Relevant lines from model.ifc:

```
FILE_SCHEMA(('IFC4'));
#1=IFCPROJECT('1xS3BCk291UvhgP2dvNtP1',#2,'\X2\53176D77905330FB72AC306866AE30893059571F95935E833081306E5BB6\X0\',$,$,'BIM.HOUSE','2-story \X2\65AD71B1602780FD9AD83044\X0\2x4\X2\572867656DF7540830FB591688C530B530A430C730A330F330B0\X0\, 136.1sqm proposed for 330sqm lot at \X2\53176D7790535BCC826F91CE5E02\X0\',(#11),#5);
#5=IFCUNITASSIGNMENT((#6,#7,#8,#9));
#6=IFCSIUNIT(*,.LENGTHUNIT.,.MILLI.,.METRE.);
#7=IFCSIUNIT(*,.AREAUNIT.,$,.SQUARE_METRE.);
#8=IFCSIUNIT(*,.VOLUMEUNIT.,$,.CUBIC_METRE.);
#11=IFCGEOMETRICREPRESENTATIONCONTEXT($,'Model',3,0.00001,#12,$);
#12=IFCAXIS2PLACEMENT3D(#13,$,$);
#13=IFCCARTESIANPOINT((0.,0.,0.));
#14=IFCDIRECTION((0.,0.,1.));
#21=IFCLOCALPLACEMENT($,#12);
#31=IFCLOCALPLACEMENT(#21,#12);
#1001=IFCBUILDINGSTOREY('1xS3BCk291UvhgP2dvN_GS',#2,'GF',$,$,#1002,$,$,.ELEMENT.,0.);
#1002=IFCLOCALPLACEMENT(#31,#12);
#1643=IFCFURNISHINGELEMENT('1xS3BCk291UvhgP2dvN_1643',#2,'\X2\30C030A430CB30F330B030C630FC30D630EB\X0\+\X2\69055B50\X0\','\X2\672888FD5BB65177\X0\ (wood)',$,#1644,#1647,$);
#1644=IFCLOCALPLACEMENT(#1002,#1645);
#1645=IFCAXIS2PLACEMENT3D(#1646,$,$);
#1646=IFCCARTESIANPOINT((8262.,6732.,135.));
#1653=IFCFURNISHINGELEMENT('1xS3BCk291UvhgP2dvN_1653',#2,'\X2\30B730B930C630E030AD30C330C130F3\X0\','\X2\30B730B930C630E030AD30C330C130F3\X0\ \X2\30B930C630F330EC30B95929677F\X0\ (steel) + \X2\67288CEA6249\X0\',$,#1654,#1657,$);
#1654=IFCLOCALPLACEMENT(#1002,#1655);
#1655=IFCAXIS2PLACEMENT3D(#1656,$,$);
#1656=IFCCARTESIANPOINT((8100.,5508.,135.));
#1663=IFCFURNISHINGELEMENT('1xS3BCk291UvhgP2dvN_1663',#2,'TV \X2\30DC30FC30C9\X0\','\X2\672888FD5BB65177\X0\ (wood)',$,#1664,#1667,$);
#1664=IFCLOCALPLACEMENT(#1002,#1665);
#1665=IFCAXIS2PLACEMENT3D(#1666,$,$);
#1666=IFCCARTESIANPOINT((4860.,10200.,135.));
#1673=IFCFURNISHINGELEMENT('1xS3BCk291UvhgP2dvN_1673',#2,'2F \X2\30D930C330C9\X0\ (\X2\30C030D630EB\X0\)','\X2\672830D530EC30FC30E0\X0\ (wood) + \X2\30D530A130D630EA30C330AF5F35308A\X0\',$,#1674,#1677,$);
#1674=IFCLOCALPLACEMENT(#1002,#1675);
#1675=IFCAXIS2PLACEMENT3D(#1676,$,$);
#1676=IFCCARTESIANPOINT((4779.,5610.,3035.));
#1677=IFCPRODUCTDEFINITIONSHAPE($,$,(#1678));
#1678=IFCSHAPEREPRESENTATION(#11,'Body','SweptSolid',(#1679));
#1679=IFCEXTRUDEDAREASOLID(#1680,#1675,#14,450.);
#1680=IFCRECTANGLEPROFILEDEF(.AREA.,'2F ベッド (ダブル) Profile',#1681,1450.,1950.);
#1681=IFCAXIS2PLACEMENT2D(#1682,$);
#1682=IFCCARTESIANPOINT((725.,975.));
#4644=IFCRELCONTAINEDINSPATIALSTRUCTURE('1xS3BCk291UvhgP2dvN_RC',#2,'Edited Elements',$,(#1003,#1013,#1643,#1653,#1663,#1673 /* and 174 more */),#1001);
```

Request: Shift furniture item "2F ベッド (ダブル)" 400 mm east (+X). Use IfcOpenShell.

```python
import ifcopenshell
import ifcopenshell.api.geometry
import ifcopenshell.util.placement

model = ifcopenshell.open("model.ifc")

item = model.by_guid("1xS3BCk291UvhgP2dvN_1673")
matrix = ifcopenshell.util.placement.get_local_placement(item.ObjectPlacement)
matrix[0, 3] += 400.0
ifcopenshell.api.geometry.edit_object_placement(model, product=item, matrix=matrix, is_si=False)

print(ifcopenshell.util.placement.get_local_placement(item.ObjectPlacement).round(3) + 0.0)

model.write("model_rev.ifc")
```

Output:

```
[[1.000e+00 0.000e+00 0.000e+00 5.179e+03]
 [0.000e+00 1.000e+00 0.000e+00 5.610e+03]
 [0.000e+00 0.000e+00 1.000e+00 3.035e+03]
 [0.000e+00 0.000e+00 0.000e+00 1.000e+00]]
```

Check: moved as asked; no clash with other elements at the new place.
